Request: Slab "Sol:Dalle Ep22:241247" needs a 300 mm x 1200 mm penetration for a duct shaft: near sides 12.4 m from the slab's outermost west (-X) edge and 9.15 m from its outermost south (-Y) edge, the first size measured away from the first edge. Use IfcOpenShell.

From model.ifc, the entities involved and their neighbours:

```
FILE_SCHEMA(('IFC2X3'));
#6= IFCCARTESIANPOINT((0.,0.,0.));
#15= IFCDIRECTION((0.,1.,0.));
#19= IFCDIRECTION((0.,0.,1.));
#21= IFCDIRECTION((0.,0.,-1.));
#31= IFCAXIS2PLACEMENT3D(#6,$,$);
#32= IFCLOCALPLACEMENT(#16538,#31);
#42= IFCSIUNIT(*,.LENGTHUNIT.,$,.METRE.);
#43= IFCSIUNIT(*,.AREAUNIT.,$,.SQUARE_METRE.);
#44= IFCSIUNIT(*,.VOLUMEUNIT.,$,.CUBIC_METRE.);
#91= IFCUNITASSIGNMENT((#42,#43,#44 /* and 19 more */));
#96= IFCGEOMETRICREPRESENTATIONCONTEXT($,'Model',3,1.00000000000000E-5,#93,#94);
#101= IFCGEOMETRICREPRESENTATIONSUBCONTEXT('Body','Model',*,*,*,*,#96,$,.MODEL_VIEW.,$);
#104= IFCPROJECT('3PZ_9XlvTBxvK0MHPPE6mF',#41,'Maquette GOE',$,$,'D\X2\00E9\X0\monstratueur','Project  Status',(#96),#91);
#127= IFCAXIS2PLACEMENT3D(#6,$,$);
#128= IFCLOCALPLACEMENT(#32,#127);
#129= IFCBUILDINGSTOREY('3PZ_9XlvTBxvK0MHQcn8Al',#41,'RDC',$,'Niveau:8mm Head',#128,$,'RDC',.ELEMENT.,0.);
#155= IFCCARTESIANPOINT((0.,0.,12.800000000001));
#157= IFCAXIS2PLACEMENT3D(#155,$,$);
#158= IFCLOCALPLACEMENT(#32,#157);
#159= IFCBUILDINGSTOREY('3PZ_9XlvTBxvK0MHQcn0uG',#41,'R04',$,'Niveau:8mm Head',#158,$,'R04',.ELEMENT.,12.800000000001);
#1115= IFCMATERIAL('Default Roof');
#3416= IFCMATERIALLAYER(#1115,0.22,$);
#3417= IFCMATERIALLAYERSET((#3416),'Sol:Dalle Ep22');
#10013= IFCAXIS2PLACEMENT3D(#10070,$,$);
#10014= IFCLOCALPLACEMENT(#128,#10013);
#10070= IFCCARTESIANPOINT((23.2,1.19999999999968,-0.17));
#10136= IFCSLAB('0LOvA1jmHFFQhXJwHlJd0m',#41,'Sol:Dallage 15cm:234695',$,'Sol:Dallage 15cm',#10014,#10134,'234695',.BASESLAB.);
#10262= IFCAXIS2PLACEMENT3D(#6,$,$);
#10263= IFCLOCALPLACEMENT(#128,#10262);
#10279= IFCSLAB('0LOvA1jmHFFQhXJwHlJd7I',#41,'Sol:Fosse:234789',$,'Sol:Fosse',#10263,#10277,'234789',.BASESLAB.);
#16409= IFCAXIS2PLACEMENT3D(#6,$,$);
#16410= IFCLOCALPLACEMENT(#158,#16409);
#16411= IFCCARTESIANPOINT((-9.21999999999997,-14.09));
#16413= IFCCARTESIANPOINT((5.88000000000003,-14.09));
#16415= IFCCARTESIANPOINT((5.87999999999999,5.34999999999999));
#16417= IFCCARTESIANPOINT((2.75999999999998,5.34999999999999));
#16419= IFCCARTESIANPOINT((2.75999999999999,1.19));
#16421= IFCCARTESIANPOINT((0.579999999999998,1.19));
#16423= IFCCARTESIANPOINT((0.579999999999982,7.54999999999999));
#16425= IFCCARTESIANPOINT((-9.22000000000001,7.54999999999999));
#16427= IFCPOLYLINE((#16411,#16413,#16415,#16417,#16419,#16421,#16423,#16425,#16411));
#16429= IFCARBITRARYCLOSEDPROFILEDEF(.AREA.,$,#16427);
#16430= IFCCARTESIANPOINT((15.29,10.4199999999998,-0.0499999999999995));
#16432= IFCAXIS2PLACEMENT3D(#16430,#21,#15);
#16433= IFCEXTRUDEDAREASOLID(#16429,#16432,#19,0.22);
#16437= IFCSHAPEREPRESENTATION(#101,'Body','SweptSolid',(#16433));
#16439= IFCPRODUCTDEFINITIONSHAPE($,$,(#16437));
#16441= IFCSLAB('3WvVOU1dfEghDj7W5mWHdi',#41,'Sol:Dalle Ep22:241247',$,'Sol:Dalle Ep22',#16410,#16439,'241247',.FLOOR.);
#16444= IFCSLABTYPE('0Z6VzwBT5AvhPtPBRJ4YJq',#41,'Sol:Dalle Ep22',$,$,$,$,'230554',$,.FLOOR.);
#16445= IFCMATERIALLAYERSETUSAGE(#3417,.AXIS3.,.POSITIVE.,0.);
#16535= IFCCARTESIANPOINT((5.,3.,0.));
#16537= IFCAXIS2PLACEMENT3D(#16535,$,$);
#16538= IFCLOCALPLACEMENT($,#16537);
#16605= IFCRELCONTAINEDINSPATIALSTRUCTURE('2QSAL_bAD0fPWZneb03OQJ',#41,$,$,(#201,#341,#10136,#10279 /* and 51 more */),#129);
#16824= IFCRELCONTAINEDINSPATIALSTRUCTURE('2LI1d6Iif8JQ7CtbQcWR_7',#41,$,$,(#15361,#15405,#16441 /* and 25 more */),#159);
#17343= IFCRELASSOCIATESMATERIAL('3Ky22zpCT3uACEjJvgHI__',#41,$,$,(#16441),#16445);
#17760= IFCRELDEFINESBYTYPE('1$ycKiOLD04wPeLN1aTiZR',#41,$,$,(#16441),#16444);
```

```python
import numpy as np
import ifcopenshell
import ifcopenshell.api.feature
import ifcopenshell.api.geometry
import ifcopenshell.api.root
import ifcopenshell.geom
import ifcopenshell.util.placement
import ifcopenshell.util.representation
import ifcopenshell.util.shape
import ifcopenshell.util.unit

model = ifcopenshell.open("model.ifc")
unit_scale = ifcopenshell.util.unit.calculate_unit_scale(model)
settings = ifcopenshell.geom.settings()


def volume(element):
    """Net volume in cubic metres, openings subtracted."""
    shape = ifcopenshell.geom.create_shape(settings, element)
    return ifcopenshell.util.shape.get_volume(shape.geometry)


slab = model.by_id(16441)
before = volume(slab)

# Extent in the slab's own axes, in metres. The edges named are its -X and -Y sides.
slab_shape = ifcopenshell.geom.create_shape(settings, slab)
vertices = ifcopenshell.util.shape.get_vertices(slab_shape.geometry)
x_min, y_min, bottom = vertices.min(axis=0)
top = vertices[:, 2].max()

opening = ifcopenshell.api.root.create_entity(model, ifc_class="IfcOpeningElement", name="Duct shaft opening")
context = ifcopenshell.util.representation.get_context(model, "Model", "Body", "MODEL_VIEW")
width, depth = 0.3, 1.2
outline = [(0.0, 0.0), (width, 0.0), (width, depth), (0.0, depth), (0.0, 0.0)]
# Overshoot both faces by 50 mm so the cut is clean.
shape = ifcopenshell.api.geometry.add_slab_representation(
    model, context=context, depth=top - bottom + 0.1, polyline=outline
)
ifcopenshell.api.geometry.assign_representation(model, product=opening, representation=shape)

matrix = ifcopenshell.util.placement.get_local_placement(slab.ObjectPlacement)
matrix[:, 3] = matrix @ np.append(np.array([x_min + 12.4, y_min + 9.15, bottom - 0.05]) / unit_scale, 1.0)
ifcopenshell.api.geometry.edit_object_placement(model, product=opening, matrix=matrix, is_si=False)
ifcopenshell.api.feature.add_feature(model, feature=opening, element=slab)

after = volume(slab)

print(f"slab volume {before:.3f} -> {after:.3f} m3")

model.write("model-out.ifc")
```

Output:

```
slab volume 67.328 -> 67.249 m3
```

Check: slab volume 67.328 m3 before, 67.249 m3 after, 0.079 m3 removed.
